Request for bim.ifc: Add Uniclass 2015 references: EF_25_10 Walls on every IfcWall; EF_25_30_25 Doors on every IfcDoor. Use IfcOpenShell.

First a look at what the model holds.

```python
import ifcopenshell

model = ifcopenshell.open("bim.ifc")
print(model.schema)
print("classifications:", [c.Name for c in model.by_type("IfcClassification")])
for ifc_class in ("IfcDoor", "IfcRoof", "IfcStair", "IfcWall", "IfcWindow"):
    print(ifc_class, len(model.by_type(ifc_class)))
```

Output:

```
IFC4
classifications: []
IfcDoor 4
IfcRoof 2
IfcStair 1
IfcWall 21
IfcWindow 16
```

```python
import ifcopenshell
import ifcopenshell.api.classification

model = ifcopenshell.open("bim.ifc")

system = ifcopenshell.api.classification.add_classification(model, classification="Uniclass 2015")

codes = {
    "IfcWall": ("EF_25_10", "Walls"),
    "IfcDoor": ("EF_25_30_25", "Doors"),
}
for ifc_class, (code, name) in codes.items():
    products = model.by_type(ifc_class)
    ifcopenshell.api.classification.add_reference(
        model, products=products, classification=system, identification=code, name=name
    )
    print(code, len(products))

model.write("bim_edited.ifc")
```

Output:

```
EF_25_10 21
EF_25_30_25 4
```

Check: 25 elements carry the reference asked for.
